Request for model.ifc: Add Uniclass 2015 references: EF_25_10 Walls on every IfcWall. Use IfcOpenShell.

First a look at what the model holds.

```python
import ifcopenshell

model = ifcopenshell.open("model.ifc")
print(model.schema)
print("classifications:", [c.Name for c in model.by_type("IfcClassification")])
for ifc_class in ("IfcDoor", "IfcRoof", "IfcStair", "IfcWall", "IfcWindow"):
    print(ifc_class, len(model.by_type(ifc_class)))
```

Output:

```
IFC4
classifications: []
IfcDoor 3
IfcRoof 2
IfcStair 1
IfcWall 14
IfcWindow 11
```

```python
import ifcopenshell
import ifcopenshell.api.classification

model = ifcopenshell.open("model.ifc")

system = ifcopenshell.api.classification.add_classification(model, classification="Uniclass 2015")

codes = {
    "IfcWall": ("EF_25_10", "Walls"),
}
for ifc_class, (code, name) in codes.items():
    products = model.by_type(ifc_class)
    ifcopenshell.api.classification.add_reference(
        model, products=products, classification=system, identification=code, name=name
    )
    print(code, len(products))

model.write("model_edited.ifc")
```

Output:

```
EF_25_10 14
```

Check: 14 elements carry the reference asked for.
